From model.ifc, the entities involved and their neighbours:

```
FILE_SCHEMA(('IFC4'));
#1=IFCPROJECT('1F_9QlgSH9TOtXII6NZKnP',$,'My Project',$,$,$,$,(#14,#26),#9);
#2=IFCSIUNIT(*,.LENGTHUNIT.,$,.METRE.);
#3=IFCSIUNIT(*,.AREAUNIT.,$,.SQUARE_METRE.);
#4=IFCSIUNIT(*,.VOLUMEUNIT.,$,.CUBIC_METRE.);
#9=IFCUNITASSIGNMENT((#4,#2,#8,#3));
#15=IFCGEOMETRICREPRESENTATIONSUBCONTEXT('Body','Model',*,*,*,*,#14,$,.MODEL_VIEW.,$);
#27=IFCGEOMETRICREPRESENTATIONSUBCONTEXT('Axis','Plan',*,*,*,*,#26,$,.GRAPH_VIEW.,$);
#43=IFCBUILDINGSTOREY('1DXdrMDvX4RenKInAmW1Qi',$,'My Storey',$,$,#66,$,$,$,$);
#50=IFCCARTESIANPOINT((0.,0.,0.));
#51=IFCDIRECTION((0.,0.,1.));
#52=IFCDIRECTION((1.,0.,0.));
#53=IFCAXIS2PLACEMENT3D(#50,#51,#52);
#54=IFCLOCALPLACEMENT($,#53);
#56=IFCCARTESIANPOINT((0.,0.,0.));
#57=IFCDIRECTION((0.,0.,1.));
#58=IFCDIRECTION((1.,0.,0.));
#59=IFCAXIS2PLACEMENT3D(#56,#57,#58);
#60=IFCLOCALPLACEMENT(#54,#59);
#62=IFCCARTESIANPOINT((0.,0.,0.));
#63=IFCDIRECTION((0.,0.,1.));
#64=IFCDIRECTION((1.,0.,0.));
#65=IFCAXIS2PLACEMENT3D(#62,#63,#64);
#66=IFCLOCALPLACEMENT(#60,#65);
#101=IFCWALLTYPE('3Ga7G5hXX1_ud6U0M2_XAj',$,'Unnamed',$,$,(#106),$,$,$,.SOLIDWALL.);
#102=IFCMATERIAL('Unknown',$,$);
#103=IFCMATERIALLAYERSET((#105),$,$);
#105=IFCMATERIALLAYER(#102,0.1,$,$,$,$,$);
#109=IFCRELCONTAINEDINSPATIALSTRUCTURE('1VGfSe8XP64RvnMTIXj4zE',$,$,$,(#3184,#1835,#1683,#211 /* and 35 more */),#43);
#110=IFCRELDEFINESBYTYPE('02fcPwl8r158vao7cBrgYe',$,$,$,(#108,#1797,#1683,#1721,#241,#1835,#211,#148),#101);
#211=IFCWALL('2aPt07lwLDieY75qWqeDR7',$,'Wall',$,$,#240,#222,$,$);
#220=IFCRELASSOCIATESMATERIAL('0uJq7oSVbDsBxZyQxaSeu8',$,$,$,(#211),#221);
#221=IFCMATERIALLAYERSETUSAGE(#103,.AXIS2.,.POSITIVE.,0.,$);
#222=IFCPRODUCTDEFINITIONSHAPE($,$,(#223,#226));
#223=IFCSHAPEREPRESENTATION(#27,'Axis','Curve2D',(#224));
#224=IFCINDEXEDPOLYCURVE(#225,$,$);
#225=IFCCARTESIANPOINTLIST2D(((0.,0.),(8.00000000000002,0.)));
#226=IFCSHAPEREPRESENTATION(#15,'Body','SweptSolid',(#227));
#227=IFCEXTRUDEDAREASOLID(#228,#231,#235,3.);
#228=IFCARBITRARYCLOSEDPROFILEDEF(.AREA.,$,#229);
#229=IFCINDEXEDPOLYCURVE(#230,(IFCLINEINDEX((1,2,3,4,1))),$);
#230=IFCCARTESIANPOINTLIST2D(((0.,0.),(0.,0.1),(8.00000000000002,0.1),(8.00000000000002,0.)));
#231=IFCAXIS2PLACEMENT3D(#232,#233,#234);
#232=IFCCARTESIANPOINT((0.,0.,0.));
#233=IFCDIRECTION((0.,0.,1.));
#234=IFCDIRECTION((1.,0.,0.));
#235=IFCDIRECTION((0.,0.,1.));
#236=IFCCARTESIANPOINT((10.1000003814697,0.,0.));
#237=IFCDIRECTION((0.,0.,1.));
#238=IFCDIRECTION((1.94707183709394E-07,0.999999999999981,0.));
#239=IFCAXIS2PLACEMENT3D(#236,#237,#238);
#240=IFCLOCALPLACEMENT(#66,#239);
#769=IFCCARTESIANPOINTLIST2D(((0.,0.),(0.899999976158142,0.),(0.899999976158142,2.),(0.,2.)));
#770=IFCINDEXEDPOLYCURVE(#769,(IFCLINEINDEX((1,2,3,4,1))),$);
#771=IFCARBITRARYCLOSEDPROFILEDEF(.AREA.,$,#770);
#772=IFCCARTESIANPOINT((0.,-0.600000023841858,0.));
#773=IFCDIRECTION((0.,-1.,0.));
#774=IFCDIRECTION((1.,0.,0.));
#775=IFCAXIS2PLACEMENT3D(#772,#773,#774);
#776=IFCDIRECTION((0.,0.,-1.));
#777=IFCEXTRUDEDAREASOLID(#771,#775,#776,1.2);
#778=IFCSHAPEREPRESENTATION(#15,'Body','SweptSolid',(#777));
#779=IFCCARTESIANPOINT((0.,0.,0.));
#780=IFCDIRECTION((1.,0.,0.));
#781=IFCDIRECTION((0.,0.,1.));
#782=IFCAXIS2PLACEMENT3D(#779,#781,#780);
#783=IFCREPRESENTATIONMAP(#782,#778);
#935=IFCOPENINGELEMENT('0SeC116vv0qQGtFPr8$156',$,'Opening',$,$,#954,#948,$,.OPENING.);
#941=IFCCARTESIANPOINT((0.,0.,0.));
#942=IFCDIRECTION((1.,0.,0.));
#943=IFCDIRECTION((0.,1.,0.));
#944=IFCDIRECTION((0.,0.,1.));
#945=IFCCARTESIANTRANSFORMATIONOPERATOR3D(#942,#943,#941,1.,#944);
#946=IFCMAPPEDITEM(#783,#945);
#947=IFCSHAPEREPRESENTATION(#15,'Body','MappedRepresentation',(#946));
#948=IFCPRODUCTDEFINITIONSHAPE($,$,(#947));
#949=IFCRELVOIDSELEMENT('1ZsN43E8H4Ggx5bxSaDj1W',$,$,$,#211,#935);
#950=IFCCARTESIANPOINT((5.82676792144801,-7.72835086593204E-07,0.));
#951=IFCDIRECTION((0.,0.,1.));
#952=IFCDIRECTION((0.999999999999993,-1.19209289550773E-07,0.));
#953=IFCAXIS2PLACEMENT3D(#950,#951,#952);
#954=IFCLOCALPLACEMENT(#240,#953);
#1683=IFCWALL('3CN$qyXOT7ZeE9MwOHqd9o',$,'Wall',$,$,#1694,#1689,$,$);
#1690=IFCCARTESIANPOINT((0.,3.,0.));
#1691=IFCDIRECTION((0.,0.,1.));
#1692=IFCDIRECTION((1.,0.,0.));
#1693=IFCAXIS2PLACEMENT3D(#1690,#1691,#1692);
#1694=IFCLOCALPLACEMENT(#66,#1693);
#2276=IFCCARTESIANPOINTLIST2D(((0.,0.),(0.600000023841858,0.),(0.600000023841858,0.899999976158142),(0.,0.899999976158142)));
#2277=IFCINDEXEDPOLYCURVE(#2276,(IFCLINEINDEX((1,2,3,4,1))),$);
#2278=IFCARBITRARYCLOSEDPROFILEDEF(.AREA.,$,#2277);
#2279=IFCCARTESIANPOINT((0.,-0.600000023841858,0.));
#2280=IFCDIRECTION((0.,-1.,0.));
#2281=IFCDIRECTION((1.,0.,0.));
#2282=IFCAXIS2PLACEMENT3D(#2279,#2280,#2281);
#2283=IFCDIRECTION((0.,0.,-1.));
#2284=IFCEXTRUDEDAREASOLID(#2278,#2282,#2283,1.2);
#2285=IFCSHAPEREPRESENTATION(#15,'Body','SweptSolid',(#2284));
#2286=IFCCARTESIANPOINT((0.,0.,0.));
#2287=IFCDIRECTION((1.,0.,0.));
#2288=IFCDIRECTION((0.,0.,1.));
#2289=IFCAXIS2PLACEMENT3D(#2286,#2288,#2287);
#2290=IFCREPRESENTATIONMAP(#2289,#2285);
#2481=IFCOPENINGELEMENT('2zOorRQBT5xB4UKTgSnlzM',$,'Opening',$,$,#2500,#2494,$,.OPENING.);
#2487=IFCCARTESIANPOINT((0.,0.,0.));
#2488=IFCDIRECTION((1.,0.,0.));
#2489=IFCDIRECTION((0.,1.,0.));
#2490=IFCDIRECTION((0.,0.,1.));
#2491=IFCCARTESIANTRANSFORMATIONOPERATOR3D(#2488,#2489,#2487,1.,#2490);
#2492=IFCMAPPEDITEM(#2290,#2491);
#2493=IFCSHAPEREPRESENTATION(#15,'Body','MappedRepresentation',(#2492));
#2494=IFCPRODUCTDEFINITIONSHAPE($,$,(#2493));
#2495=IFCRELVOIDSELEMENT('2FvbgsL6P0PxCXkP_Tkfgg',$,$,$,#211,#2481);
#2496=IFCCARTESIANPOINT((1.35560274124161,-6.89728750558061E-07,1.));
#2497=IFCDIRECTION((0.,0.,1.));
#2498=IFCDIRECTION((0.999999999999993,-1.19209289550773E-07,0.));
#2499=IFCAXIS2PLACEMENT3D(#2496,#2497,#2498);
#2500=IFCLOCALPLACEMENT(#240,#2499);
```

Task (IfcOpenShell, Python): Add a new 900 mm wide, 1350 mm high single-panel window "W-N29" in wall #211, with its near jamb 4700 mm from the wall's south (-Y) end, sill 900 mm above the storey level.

```python
import numpy as np
import ifcopenshell
import ifcopenshell.api.feature
import ifcopenshell.api.geometry
import ifcopenshell.api.root
import ifcopenshell.api.spatial
import ifcopenshell.geom
import ifcopenshell.util.element
import ifcopenshell.util.placement
import ifcopenshell.util.representation
import ifcopenshell.util.shape
import ifcopenshell.util.unit

model = ifcopenshell.open("model.ifc")
unit_scale = ifcopenshell.util.unit.calculate_unit_scale(model)
settings = ifcopenshell.geom.settings()


def volume(element):
    """Net volume in cubic metres, openings subtracted."""
    shape = ifcopenshell.geom.create_shape(settings, element)
    return ifcopenshell.util.shape.get_volume(shape.geometry)


wall = model.by_id(211)
storey = ifcopenshell.util.element.get_container(wall, ifc_class="IfcBuildingStorey")
context = ifcopenshell.util.representation.get_context(model, "Model", "Body", "MODEL_VIEW")
before = volume(wall)

width, height, from_end, sill = 0.9, 1.35, 4.7, 0.9  # metres

# The wall runs along its own X axis, and the end named is its -X end.
wall_shape = ifcopenshell.geom.create_shape(settings, wall)
x, y, z = ifcopenshell.util.shape.get_vertices(wall_shape.geometry).T
start = x.min() + from_end
face, thickness = float(y.min()), float(y.max() - y.min())
wall_matrix = ifcopenshell.util.placement.get_local_placement(wall.ObjectPlacement)
level = ifcopenshell.util.placement.get_local_placement(storey.ObjectPlacement)[2, 3]


def in_wall(x, y):
    """Placement at x, y metres in the wall's axes, at sill height."""
    matrix = wall_matrix.copy()
    matrix[:, 3] = wall_matrix @ np.array([x / unit_scale, y / unit_scale, 0.0, 1.0])
    matrix[2, 3] = level + sill / unit_scale
    return matrix


# Opening: a box that overshoots both wall faces by 50 mm.
opening = ifcopenshell.api.root.create_entity(model, ifc_class="IfcOpeningElement", predefined_type="OPENING")
box = ifcopenshell.api.geometry.add_wall_representation(
    model, context=context, length=width, height=height, thickness=thickness + 0.1
)
ifcopenshell.api.geometry.assign_representation(model, product=opening, representation=box)
ifcopenshell.api.geometry.edit_object_placement(model, product=opening, matrix=in_wall(start, face - 0.05), is_si=False)
ifcopenshell.api.feature.add_feature(model, feature=opening, element=wall)

window = ifcopenshell.api.root.create_entity(model, ifc_class="IfcWindow", name="W-N29", predefined_type="WINDOW")
window.OverallWidth, window.OverallHeight = width / unit_scale, height / unit_scale
window.PartitioningType = "SINGLE_PANEL"
body = ifcopenshell.api.geometry.add_window_representation(
    model,
    context=context,
    overall_width=window.OverallWidth,
    overall_height=window.OverallHeight,
    partition_type="SINGLE_PANEL",
)
ifcopenshell.api.geometry.assign_representation(model, product=window, representation=body)
ifcopenshell.api.spatial.assign_container(model, products=[window], relating_structure=storey)
ifcopenshell.api.feature.add_filling(model, opening=opening, element=window)

# Centre the window in the wall's thickness.
ifcopenshell.api.geometry.edit_object_placement(model, product=window, matrix=in_wall(start, face), is_si=False)
window_shape = ifcopenshell.geom.create_shape(settings, window)
depth = ifcopenshell.util.shape.get_vertices(window_shape.geometry)[:, 1]
offset = face + thickness / 2 - (depth.min() + depth.max()) / 2
ifcopenshell.api.geometry.edit_object_placement(model, product=window, matrix=in_wall(start, offset), is_si=False)

after = volume(wall)

print(f"wall volume {before:.3f} -> {after:.3f} m3")

model.write("model-out.ifc")
```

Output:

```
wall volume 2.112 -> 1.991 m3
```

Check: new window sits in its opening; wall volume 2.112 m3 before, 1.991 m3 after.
